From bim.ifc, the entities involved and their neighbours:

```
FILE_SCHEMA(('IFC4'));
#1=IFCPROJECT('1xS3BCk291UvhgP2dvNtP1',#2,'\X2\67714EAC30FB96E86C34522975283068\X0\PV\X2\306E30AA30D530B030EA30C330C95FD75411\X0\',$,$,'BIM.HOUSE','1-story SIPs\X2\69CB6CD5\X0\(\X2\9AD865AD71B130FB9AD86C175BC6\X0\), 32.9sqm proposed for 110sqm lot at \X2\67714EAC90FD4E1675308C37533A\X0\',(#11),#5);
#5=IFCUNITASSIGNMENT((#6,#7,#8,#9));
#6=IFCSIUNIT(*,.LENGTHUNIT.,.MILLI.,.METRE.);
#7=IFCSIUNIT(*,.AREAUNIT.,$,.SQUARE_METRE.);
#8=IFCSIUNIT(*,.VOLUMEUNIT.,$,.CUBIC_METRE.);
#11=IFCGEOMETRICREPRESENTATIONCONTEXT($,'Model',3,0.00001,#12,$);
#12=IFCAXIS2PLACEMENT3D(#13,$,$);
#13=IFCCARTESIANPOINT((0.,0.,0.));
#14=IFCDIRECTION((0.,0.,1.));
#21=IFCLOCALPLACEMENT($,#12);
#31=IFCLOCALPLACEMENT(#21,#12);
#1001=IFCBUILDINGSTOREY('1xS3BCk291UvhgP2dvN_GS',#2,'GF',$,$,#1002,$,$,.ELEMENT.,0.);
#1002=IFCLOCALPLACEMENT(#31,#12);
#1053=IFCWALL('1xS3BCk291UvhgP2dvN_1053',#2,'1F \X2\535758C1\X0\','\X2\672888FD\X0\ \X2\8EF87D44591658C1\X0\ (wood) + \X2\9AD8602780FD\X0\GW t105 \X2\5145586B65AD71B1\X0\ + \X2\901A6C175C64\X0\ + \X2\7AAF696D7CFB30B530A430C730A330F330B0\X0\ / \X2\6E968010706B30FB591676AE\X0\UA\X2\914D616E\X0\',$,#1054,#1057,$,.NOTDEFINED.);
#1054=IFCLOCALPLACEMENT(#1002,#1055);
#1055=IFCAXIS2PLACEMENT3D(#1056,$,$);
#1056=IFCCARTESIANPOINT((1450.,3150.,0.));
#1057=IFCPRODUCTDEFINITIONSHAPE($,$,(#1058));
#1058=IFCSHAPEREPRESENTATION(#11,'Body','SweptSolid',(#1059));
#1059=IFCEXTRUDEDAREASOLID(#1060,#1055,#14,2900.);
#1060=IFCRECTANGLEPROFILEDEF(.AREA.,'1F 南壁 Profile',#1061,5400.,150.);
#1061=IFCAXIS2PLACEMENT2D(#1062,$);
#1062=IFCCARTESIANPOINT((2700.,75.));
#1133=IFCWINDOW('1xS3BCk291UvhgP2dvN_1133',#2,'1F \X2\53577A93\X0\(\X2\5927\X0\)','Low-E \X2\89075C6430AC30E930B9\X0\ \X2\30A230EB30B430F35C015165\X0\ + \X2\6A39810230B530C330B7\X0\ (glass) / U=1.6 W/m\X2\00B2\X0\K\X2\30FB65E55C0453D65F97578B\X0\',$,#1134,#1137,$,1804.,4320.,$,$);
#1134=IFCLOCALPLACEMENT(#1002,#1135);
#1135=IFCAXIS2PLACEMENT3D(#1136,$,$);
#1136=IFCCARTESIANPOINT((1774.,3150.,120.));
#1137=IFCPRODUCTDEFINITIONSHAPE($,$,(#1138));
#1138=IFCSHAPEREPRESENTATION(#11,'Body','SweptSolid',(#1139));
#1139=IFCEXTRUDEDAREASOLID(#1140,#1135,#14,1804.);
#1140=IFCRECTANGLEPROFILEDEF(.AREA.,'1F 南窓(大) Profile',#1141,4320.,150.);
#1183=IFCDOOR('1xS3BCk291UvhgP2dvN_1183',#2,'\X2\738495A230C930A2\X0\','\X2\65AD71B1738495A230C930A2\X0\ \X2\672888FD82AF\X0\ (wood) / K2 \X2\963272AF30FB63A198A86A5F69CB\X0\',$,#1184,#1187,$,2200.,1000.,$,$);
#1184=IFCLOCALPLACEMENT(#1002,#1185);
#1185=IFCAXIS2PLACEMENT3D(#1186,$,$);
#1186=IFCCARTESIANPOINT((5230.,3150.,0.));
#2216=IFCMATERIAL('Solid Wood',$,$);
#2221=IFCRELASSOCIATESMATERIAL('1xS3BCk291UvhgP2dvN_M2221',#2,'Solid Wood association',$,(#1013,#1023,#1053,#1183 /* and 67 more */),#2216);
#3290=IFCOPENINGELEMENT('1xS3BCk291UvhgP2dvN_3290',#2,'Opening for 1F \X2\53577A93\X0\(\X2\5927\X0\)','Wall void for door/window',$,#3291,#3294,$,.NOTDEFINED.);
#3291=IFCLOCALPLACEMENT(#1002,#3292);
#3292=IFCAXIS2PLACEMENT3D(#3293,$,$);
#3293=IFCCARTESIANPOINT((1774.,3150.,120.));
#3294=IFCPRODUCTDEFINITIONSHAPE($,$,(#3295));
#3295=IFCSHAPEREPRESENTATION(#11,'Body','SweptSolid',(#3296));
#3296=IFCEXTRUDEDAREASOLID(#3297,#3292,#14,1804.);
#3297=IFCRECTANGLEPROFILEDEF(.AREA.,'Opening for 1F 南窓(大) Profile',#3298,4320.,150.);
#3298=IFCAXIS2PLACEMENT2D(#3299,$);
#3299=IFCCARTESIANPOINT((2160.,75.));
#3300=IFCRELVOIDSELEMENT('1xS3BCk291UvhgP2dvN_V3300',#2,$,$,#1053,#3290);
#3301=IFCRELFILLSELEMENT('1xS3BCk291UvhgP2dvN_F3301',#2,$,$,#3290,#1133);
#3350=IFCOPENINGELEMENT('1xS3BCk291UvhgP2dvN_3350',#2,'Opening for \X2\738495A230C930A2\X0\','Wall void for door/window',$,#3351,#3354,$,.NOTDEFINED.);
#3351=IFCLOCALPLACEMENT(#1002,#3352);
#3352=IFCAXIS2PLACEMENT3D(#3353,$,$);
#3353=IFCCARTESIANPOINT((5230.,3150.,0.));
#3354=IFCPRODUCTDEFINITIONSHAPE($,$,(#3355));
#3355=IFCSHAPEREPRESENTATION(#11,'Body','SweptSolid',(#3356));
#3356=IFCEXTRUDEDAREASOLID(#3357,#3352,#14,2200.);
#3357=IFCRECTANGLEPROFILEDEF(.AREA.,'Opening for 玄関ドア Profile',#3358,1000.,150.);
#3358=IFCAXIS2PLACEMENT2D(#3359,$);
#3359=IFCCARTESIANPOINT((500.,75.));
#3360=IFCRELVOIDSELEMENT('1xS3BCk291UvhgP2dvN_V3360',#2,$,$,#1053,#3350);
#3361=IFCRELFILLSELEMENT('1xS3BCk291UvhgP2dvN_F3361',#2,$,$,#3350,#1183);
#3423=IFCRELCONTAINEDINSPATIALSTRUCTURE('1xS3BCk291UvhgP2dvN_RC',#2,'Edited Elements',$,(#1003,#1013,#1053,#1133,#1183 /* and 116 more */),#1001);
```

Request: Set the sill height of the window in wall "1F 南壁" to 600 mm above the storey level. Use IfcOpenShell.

```python
import numpy as np
import ifcopenshell
import ifcopenshell.api.geometry
import ifcopenshell.geom
import ifcopenshell.util.element
import ifcopenshell.util.placement
import ifcopenshell.util.shape
import ifcopenshell.util.unit

model = ifcopenshell.open("bim.ifc")
unit_scale = ifcopenshell.util.unit.calculate_unit_scale(model)

window = model.by_guid("1xS3BCk291UvhgP2dvN_1133")
opening = window.FillsVoids[0].RelatingOpeningElement
storey = ifcopenshell.util.element.get_container(window, ifc_class="IfcBuildingStorey")
level = ifcopenshell.util.placement.get_local_placement(storey.ObjectPlacement)[2, 3]

# The opening's origin need not be at the sill, so measure its lowest point.
shape = ifcopenshell.geom.create_shape(ifcopenshell.geom.settings(), opening)
bottom = ifcopenshell.util.shape.get_shape_bottom_elevation(shape, shape.geometry) / unit_scale
dz = level + 0.6 / unit_scale - bottom

shift = np.array([0.0, 0.0, dz])
# The window is not placed relative to its opening, so move both.
for product in (opening, window):
    matrix = ifcopenshell.util.placement.get_local_placement(product.ObjectPlacement)
    matrix[:3, 3] += shift
    ifcopenshell.api.geometry.edit_object_placement(model, product=product, matrix=matrix, is_si=False)

print(f"moved by {dz * unit_scale:+.3f} m")

model.write("bim_rev.ifc")
```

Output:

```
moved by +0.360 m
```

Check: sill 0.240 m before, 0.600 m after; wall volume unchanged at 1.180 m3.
